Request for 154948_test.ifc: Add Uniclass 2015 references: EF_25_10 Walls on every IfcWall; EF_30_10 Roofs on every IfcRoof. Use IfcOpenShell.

First a look at what the model holds.

```python
import ifcopenshell

model = ifcopenshell.open("154948_test.ifc")
print(model.schema)
print("classifications:", [c.Name for c in model.by_type("IfcClassification")])
for ifc_class in ("IfcDoor", "IfcRoof", "IfcStair", "IfcWall", "IfcWindow"):
    print(ifc_class, len(model.by_type(ifc_class)))
```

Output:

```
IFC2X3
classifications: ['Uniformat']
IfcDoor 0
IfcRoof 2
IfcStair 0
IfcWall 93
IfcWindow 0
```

```python
import ifcopenshell
import ifcopenshell.api.classification

model = ifcopenshell.open("154948_test.ifc")

# IFC2X3 requires Source and Edition and has no link from the project to the system.
system = model.create_entity("IfcClassification", Source="NBS", Edition="2015", Name="Uniclass 2015")

codes = {
    "IfcWall": ("EF_25_10", "Walls"),
    "IfcRoof": ("EF_30_10", "Roofs"),
}
for ifc_class, (code, name) in codes.items():
    products = model.by_type(ifc_class)
    ifcopenshell.api.classification.add_reference(
        model, products=products, classification=system, identification=code, name=name
    )
    print(code, len(products))

model.write("154948_test-out.ifc")
```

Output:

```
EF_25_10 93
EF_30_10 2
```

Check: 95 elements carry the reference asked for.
